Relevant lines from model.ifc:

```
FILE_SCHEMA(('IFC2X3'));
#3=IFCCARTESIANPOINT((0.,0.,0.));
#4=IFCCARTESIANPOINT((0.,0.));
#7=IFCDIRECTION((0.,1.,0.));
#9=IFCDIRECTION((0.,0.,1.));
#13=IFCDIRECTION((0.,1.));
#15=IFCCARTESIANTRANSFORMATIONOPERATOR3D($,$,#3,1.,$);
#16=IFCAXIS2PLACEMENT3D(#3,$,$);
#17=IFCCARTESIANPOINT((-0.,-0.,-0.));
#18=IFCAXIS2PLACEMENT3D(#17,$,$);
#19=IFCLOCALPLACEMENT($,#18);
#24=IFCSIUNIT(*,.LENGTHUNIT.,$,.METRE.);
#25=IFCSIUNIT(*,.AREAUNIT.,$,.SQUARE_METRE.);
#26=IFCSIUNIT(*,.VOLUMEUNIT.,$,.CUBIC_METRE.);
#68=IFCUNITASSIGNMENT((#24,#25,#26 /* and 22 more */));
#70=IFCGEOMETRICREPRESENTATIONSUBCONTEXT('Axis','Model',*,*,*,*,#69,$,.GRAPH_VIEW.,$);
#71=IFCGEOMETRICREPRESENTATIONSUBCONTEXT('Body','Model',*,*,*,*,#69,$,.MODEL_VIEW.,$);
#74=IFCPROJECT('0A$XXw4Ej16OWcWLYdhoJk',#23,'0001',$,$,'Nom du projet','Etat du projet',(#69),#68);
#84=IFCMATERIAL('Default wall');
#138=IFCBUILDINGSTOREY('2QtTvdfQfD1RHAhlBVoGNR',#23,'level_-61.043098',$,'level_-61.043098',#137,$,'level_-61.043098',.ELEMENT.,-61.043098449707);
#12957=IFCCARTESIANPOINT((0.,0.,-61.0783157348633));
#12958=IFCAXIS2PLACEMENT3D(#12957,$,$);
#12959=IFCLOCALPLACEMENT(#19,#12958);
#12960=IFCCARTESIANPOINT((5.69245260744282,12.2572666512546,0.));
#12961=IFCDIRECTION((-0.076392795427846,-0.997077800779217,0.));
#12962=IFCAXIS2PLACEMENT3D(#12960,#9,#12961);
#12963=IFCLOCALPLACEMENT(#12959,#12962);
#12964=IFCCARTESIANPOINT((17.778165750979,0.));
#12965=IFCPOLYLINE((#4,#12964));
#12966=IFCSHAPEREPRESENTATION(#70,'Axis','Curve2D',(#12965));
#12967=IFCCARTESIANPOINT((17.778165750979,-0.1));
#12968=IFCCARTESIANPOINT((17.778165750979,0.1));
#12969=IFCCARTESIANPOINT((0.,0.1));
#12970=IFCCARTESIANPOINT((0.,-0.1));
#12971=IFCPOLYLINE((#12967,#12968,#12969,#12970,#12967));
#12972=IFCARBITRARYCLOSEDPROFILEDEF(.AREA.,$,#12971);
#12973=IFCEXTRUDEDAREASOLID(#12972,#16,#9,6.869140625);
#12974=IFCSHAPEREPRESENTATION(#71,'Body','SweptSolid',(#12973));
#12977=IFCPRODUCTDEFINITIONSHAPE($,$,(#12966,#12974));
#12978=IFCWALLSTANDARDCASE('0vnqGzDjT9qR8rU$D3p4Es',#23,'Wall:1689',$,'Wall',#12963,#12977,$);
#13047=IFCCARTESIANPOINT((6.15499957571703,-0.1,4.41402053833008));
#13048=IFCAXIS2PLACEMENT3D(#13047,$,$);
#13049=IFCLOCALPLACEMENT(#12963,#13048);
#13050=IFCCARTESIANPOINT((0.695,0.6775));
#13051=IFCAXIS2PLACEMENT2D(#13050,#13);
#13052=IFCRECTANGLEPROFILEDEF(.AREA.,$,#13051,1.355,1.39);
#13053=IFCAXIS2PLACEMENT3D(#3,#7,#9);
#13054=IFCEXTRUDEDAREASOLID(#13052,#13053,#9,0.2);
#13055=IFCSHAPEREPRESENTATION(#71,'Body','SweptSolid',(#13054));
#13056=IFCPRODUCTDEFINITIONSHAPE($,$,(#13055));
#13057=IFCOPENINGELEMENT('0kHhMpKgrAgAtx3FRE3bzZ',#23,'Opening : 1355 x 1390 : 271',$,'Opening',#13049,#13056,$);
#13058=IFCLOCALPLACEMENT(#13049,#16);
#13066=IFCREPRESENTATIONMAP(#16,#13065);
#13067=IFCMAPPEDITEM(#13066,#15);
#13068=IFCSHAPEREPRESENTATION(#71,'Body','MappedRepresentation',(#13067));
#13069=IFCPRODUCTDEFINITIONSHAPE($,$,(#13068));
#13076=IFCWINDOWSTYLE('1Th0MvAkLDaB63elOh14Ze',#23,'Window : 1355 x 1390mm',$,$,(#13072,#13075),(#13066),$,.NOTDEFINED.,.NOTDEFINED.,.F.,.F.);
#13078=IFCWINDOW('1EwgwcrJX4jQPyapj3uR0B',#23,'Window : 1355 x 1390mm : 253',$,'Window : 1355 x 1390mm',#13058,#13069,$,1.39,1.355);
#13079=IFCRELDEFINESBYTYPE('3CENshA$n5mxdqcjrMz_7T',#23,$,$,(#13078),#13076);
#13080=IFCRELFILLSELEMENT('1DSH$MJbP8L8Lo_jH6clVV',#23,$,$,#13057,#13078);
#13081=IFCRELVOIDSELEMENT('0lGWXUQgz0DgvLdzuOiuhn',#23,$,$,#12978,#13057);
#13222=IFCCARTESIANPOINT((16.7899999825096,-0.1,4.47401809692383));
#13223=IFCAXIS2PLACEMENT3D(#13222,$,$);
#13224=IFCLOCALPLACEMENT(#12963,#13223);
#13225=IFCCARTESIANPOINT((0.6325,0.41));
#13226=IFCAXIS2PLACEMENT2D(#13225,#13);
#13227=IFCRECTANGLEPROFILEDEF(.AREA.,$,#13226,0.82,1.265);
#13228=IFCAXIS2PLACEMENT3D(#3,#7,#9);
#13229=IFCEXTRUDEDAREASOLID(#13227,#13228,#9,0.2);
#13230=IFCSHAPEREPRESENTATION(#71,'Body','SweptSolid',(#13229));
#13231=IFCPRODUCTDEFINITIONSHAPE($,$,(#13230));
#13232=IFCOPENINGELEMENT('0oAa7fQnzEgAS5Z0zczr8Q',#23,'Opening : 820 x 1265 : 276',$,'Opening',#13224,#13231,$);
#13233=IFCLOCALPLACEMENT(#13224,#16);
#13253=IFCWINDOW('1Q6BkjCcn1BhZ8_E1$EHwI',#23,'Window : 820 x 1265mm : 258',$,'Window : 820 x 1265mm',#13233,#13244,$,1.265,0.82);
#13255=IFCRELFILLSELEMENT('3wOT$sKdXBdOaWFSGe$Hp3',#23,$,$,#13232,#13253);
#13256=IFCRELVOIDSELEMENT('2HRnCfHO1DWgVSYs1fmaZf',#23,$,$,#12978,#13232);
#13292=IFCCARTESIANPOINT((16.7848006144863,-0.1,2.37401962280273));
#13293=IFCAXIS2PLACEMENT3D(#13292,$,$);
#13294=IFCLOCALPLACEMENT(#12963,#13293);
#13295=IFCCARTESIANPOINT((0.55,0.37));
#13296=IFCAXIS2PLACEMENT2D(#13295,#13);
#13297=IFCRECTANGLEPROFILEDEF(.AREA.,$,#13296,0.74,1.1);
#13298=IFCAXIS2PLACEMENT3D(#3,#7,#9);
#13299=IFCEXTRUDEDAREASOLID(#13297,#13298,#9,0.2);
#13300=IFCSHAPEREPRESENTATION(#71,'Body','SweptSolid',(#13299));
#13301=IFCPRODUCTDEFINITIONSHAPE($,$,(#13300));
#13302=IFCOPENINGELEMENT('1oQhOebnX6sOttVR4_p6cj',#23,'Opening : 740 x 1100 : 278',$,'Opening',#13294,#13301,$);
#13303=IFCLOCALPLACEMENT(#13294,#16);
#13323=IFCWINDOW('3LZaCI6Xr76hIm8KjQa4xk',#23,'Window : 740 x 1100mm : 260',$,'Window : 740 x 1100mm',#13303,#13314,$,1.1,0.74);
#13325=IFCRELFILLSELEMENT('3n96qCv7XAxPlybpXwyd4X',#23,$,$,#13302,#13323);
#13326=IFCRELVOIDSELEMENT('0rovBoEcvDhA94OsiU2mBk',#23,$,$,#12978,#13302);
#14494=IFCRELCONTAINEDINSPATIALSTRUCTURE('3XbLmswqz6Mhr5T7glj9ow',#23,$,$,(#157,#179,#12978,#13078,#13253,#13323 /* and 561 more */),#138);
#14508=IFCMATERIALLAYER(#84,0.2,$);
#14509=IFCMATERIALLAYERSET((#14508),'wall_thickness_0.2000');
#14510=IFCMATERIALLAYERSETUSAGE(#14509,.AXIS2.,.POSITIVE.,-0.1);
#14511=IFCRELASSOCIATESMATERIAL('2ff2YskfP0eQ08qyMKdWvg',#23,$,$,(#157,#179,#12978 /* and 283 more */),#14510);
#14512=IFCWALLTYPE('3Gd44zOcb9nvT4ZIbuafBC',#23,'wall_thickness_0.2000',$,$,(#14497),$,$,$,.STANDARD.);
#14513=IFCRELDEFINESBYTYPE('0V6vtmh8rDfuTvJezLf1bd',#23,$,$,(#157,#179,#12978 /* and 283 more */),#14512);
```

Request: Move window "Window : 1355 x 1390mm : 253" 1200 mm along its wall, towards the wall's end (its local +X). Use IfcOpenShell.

```python
import ifcopenshell
import ifcopenshell.api.geometry
import ifcopenshell.util.placement

model = ifcopenshell.open("model.ifc")

window = model.by_guid("1EwgwcrJX4jQPyapj3uR0B")
opening = window.FillsVoids[0].RelatingOpeningElement
wall = opening.VoidsElements[0].RelatingBuildingElement

wall_matrix = ifcopenshell.util.placement.get_local_placement(wall.ObjectPlacement)
shift = wall_matrix[:3, 0] * 1.2
before = ifcopenshell.util.placement.get_local_placement(window.ObjectPlacement)[:3, 3].copy()

# The window is placed relative to its opening, so it follows when the opening moves.
matrix = ifcopenshell.util.placement.get_local_placement(opening.ObjectPlacement)
matrix[:3, 3] += shift
ifcopenshell.api.geometry.edit_object_placement(
    model, product=opening, matrix=matrix, is_si=False, should_transform_children=True
)

after = ifcopenshell.util.placement.get_local_placement(window.ObjectPlacement)[:3, 3]
print("window moved by", (after - before).round(3) + 0.0)

model.write("model_edited.ifc")
```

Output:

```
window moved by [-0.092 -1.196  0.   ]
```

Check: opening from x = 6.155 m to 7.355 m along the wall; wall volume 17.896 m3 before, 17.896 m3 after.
